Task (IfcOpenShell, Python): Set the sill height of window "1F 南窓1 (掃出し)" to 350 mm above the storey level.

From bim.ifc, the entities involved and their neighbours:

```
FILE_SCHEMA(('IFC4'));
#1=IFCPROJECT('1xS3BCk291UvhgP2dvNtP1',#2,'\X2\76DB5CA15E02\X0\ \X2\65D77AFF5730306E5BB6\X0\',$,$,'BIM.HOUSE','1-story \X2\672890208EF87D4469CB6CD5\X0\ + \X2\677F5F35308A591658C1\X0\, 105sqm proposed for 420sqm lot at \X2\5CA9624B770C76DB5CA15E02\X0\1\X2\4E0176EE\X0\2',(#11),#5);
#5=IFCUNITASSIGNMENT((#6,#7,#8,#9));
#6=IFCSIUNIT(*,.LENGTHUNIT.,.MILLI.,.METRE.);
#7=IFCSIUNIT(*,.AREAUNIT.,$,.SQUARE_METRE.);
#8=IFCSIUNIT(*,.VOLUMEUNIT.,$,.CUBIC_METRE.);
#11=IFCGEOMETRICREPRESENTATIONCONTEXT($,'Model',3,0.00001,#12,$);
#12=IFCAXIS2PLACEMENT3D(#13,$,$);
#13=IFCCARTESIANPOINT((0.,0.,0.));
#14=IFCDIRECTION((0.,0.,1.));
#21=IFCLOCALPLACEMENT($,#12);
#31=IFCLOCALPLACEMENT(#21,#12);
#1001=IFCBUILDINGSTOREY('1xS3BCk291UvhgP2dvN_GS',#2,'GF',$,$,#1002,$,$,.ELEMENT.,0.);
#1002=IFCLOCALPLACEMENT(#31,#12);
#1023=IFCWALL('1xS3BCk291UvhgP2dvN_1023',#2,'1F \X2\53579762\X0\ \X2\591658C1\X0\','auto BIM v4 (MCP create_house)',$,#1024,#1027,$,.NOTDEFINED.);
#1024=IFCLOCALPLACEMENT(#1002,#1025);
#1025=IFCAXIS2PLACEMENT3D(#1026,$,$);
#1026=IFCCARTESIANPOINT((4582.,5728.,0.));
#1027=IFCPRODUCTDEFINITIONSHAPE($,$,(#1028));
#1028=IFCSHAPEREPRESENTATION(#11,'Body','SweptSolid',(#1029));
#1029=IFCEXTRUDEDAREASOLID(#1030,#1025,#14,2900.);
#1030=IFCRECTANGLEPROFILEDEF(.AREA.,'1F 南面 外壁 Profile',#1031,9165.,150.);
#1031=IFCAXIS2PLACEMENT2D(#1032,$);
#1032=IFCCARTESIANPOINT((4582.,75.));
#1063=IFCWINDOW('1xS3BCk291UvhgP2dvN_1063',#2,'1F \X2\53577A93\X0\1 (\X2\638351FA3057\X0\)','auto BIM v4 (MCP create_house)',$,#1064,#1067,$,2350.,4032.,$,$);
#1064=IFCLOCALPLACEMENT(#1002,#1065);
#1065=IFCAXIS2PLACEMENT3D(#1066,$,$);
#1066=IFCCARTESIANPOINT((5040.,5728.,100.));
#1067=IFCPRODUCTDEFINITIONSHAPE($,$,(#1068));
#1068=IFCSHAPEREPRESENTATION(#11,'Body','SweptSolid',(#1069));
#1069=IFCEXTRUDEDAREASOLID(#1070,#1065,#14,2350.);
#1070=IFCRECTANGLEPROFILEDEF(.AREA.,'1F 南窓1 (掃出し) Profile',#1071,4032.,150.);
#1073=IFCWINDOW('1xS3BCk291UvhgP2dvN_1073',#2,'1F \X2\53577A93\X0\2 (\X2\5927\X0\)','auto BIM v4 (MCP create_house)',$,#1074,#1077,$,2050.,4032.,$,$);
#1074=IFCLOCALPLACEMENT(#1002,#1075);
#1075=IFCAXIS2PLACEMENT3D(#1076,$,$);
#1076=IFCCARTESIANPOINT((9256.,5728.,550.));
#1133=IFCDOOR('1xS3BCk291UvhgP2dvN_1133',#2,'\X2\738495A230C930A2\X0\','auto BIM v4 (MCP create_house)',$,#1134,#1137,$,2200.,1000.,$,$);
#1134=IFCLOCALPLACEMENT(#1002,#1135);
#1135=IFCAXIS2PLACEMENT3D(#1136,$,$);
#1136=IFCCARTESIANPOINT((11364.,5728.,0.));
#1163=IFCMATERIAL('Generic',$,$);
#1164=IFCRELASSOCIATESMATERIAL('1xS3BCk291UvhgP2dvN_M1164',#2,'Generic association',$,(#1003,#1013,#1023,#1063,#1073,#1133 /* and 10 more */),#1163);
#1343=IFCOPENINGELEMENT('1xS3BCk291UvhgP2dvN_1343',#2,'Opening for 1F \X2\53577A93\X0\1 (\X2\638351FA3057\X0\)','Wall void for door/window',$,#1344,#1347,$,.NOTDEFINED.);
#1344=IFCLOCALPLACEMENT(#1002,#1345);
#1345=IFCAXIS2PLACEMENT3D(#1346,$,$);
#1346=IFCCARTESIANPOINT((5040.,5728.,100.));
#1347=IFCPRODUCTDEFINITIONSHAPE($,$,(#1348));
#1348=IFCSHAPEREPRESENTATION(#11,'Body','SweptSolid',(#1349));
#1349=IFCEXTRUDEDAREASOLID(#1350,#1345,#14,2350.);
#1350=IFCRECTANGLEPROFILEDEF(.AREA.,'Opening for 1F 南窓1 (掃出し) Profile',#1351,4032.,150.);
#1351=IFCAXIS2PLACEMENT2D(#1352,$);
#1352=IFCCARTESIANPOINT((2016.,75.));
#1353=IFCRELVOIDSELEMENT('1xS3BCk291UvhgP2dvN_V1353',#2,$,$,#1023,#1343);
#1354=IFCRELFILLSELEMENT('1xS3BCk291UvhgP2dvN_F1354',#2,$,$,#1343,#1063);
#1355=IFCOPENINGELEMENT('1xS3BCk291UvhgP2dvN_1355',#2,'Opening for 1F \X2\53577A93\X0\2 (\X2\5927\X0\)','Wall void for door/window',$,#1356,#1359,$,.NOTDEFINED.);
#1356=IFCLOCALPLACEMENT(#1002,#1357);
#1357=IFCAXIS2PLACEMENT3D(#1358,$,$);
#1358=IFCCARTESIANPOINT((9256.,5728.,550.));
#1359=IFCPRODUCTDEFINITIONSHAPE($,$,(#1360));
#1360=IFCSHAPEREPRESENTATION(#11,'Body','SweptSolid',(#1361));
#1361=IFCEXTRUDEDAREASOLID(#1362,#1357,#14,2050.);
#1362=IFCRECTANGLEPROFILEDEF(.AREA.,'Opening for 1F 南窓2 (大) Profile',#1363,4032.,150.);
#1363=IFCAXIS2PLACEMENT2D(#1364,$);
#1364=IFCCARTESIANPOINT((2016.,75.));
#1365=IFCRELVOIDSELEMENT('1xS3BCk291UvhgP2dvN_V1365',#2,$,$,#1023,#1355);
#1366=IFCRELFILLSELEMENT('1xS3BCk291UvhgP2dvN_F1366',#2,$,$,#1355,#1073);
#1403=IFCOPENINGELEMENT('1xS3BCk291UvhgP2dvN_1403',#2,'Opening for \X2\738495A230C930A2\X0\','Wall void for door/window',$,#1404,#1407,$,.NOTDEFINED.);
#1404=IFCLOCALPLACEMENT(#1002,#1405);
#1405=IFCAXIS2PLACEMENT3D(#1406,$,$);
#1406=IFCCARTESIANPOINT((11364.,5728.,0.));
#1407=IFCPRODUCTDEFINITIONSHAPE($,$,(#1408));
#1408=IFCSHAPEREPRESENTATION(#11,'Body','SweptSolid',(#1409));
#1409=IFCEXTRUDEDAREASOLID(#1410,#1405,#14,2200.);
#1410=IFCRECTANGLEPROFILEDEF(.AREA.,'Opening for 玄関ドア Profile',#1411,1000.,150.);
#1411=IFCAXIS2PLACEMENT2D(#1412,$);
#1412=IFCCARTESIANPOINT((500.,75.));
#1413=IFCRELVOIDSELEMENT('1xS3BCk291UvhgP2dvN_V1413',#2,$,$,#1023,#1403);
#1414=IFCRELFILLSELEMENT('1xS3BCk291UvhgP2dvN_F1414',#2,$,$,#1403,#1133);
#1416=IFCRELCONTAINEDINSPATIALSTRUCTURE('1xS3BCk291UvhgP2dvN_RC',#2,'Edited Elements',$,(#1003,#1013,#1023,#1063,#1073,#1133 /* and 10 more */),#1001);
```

```python
import numpy as np
import ifcopenshell
import ifcopenshell.api.geometry
import ifcopenshell.geom
import ifcopenshell.util.element
import ifcopenshell.util.placement
import ifcopenshell.util.shape
import ifcopenshell.util.unit

model = ifcopenshell.open("bim.ifc")
unit_scale = ifcopenshell.util.unit.calculate_unit_scale(model)

window = model.by_guid("1xS3BCk291UvhgP2dvN_1063")
opening = window.FillsVoids[0].RelatingOpeningElement
storey = ifcopenshell.util.element.get_container(window, ifc_class="IfcBuildingStorey")
level = ifcopenshell.util.placement.get_local_placement(storey.ObjectPlacement)[2, 3]

# The opening's origin need not be at the sill, so measure its lowest point.
shape = ifcopenshell.geom.create_shape(ifcopenshell.geom.settings(), opening)
bottom = ifcopenshell.util.shape.get_shape_bottom_elevation(shape, shape.geometry) / unit_scale
dz = level + 0.35 / unit_scale - bottom

shift = np.array([0.0, 0.0, dz])
# The window is not placed relative to its opening, so move both.
for product in (opening, window):
    matrix = ifcopenshell.util.placement.get_local_placement(product.ObjectPlacement)
    matrix[:3, 3] += shift
    ifcopenshell.api.geometry.edit_object_placement(model, product=product, matrix=matrix, is_si=False)

print(f"moved by {dz * unit_scale:+.3f} m")

model.write("bim_edited.ifc")
```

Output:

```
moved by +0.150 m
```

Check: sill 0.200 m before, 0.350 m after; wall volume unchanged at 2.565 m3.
